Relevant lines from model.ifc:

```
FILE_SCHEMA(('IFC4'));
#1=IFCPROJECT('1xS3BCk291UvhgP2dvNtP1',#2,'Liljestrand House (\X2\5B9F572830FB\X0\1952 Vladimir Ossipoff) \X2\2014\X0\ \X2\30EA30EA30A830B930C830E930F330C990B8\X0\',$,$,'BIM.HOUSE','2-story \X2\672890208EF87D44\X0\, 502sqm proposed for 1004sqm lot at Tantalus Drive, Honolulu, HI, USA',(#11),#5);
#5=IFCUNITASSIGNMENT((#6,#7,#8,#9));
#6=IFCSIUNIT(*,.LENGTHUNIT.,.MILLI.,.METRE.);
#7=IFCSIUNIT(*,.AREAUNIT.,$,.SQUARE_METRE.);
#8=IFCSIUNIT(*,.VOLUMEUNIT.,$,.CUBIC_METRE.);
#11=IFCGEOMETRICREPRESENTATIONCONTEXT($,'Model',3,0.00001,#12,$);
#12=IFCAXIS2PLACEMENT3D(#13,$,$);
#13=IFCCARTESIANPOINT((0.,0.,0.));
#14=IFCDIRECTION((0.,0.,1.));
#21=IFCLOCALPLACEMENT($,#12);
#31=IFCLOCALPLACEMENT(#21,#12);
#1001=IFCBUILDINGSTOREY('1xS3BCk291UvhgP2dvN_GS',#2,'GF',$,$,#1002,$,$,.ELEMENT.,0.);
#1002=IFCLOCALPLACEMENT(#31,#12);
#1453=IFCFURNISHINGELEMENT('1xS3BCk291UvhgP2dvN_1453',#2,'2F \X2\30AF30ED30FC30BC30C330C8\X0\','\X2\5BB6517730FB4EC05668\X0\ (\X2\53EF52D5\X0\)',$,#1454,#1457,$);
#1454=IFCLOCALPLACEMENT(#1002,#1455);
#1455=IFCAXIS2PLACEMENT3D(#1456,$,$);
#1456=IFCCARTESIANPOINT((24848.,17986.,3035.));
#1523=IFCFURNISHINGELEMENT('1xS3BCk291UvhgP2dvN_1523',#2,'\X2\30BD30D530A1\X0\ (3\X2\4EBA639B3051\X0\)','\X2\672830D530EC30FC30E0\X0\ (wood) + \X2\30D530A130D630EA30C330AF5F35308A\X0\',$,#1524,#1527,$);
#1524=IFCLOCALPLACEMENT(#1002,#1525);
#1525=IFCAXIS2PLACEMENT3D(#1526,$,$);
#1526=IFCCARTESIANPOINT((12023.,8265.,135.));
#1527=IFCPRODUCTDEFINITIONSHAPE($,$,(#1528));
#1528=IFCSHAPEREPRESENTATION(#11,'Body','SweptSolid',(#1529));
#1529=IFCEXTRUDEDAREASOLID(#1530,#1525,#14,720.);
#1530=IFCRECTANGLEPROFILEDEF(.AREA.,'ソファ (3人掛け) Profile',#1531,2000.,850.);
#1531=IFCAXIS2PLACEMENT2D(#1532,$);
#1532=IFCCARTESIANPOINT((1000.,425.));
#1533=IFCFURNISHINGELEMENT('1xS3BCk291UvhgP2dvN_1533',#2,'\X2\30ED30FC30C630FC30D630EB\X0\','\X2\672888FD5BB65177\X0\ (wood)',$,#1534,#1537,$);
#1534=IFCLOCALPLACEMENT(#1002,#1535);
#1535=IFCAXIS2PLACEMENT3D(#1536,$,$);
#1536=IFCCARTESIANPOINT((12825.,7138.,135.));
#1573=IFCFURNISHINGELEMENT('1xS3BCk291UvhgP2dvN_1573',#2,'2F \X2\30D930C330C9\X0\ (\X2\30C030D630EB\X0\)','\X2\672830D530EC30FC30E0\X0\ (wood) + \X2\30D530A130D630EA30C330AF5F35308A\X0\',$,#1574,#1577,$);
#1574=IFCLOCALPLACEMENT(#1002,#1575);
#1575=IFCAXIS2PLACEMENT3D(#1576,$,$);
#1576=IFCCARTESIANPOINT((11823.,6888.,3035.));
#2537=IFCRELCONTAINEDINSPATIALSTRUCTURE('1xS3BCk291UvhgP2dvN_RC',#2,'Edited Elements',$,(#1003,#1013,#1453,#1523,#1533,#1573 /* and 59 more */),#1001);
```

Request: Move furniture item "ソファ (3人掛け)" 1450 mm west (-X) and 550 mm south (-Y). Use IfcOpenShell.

```python
import ifcopenshell
import ifcopenshell.api.geometry
import ifcopenshell.util.placement
import ifcopenshell.util.unit

model = ifcopenshell.open("model.ifc")
unit_scale = ifcopenshell.util.unit.calculate_unit_scale(model)

item = model.by_guid("1xS3BCk291UvhgP2dvN_1523")
matrix = ifcopenshell.util.placement.get_local_placement(item.ObjectPlacement)
matrix[0, 3] -= 1.45 / unit_scale
matrix[1, 3] -= 0.55 / unit_scale
ifcopenshell.api.geometry.edit_object_placement(model, product=item, matrix=matrix, is_si=False)

print(ifcopenshell.util.placement.get_local_placement(item.ObjectPlacement).round(3) + 0.0)

model.write("model_updated.ifc")
```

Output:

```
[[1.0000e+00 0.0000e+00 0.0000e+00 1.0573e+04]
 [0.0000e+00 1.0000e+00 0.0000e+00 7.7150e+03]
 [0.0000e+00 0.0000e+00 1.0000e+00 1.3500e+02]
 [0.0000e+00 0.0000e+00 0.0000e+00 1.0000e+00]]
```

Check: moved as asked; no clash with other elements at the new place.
